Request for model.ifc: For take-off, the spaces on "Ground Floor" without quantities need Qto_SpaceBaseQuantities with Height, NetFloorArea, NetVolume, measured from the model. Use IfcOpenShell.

First a look at what the model holds.

```python
import ifcopenshell
import ifcopenshell.util.element
import ifcopenshell.util.unit

model = ifcopenshell.open("model.ifc")
print(model.schema)
for unit_type in ("LENGTHUNIT", "AREAUNIT", "VOLUMEUNIT"):
    print(unit_type, ifcopenshell.util.unit.calculate_unit_scale(model, unit_type))
storey = next(s for s in model.by_type("IfcBuildingStorey") if s.Name == "Ground Floor")
spaces = [e for e in ifcopenshell.util.element.get_decomposition(storey) if e.is_a("IfcSpace")]
for e in sorted(spaces, key=lambda e: e.id()):
    print(e.id(), e.is_a(), e.Name, list(ifcopenshell.util.element.get_psets(e, qtos_only=True)), sep=" | ")
```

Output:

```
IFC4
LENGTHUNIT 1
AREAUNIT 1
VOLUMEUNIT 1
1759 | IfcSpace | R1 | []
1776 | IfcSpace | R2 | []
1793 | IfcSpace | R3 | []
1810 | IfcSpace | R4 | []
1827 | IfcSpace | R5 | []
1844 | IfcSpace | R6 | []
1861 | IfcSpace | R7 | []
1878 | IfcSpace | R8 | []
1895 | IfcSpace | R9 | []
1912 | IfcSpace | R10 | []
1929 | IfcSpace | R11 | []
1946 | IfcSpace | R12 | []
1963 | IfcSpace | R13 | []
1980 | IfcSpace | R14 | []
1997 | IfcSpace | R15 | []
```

```python
import ifcopenshell
import ifcopenshell.api.pset
import ifcopenshell.geom
import ifcopenshell.util.element
import ifcopenshell.util.shape
import ifcopenshell.util.unit

model = ifcopenshell.open("model.ifc")
unit_scale = ifcopenshell.util.unit.calculate_unit_scale(model)
area_scale = ifcopenshell.util.unit.calculate_unit_scale(model, "AREAUNIT")
volume_scale = ifcopenshell.util.unit.calculate_unit_scale(model, "VOLUMEUNIT")
settings = ifcopenshell.geom.settings()

storey = next(s for s in model.by_type("IfcBuildingStorey") if s.Name == "Ground Floor")
spaces = [e for e in ifcopenshell.util.element.get_decomposition(storey) if e.is_a("IfcSpace")]

for e in sorted(spaces, key=lambda e: e.id()):
    if ifcopenshell.util.element.get_psets(e, qtos_only=True, should_inherit=False):
        continue
    # Geometry comes back in metres, in the element's own axes.
    shape = ifcopenshell.geom.create_shape(settings, e)
    values = {
        "Height": ifcopenshell.util.shape.get_z(shape.geometry) / unit_scale,
        "NetFloorArea": ifcopenshell.util.shape.get_footprint_area(shape.geometry) / area_scale,
        "NetVolume": ifcopenshell.util.shape.get_volume(shape.geometry) / volume_scale,
    }
    qto = ifcopenshell.api.pset.add_qto(model, product=e, name="Qto_SpaceBaseQuantities")
    ifcopenshell.api.pset.edit_qto(model, qto=qto, properties=values)
    print(e.id(), {k: round(v, 3) for k, v in values.items()})

model.write("model_updated.ifc")
```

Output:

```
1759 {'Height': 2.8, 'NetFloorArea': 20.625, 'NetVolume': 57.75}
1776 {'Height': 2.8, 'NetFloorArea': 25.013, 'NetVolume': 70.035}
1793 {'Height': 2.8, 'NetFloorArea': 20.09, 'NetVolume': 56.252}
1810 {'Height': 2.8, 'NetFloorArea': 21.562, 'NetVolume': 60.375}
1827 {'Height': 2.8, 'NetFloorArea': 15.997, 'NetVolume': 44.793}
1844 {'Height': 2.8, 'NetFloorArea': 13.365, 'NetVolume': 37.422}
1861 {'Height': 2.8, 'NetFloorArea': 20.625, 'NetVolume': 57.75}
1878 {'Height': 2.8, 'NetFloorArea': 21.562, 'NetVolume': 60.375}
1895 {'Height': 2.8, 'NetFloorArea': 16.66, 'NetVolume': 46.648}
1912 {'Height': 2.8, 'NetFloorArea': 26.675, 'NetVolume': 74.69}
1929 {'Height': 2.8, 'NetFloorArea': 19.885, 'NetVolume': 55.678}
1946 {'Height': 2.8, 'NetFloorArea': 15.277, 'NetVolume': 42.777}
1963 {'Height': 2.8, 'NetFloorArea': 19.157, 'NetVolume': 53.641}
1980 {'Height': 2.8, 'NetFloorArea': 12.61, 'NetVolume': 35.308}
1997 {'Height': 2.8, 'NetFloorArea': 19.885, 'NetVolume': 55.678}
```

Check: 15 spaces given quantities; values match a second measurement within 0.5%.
